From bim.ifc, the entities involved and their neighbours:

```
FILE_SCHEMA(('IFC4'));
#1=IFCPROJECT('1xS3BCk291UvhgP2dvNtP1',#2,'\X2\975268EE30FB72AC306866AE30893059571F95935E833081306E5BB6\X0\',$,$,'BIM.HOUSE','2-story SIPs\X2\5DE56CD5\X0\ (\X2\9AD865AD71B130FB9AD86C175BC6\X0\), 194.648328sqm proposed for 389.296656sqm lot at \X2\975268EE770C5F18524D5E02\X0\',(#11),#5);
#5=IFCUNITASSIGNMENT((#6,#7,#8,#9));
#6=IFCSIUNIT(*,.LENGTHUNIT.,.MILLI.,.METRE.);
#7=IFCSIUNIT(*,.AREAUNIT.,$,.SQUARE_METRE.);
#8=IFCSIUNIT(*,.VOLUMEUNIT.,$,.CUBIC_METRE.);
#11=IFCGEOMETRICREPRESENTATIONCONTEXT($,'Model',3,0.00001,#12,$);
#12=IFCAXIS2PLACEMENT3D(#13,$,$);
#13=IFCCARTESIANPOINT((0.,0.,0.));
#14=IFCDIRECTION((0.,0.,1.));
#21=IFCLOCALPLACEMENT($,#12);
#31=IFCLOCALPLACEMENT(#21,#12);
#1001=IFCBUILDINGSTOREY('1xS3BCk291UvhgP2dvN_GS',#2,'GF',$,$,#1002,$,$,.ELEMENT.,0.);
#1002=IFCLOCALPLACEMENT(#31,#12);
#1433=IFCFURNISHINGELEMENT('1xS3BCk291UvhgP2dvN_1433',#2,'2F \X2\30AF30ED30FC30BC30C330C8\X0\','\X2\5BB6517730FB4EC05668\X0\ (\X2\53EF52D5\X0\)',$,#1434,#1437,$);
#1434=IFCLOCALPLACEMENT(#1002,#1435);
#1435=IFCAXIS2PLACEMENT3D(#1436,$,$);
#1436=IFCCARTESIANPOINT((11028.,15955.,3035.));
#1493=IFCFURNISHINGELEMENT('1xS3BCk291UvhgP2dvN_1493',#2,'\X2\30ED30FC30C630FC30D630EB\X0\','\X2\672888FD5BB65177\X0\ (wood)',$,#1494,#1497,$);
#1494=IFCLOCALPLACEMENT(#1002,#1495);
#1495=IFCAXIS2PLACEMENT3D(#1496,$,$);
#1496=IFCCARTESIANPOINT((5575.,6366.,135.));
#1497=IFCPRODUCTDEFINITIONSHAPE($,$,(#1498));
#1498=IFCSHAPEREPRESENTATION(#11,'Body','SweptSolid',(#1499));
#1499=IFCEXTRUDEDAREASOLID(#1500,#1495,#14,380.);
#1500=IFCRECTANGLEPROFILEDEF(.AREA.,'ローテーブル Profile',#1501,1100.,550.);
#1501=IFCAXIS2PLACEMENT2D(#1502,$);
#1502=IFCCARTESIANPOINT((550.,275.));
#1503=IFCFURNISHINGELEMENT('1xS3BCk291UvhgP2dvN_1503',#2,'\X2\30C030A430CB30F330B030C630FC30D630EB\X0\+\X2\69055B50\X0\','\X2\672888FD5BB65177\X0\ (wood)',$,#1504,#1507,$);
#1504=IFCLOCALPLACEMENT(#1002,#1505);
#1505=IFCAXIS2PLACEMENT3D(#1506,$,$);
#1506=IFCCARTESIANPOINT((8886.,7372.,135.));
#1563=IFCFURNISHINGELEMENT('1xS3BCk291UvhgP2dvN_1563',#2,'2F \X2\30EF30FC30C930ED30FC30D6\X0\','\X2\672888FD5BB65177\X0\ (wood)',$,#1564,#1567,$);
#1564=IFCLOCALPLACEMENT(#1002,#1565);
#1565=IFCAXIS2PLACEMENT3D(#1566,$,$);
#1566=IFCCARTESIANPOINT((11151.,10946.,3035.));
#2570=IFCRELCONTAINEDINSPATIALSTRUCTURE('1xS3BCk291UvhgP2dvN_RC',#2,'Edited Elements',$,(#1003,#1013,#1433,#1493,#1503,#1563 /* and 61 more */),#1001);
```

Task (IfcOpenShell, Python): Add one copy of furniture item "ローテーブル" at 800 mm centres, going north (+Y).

```python
import numpy as np
import ifcopenshell
import ifcopenshell.api.geometry
import ifcopenshell.api.root
import ifcopenshell.util.element
import ifcopenshell.util.placement
import ifcopenshell.util.unit

model = ifcopenshell.open("bim.ifc")
unit_scale = ifcopenshell.util.unit.calculate_unit_scale(model)


def reuse_history(source, copy):
    """copy_class also copies each property set's owner history, people and application; keep the originals."""
    for rel in copy.IsDefinedBy:
        if rel.is_a("IfcRelDefinesByProperties") and (history := rel.RelatingPropertyDefinition.OwnerHistory):
            rel.RelatingPropertyDefinition.OwnerHistory = source.OwnerHistory
            ifcopenshell.util.element.remove_deep2(model, history)


source = model.by_guid("1xS3BCk291UvhgP2dvN_1493")
base = ifcopenshell.util.placement.get_local_placement(source.ObjectPlacement)
step = np.array([0.0, 1.0, 0.0]) * 0.8 / unit_scale

for i in range(1, 2):
    copy = ifcopenshell.api.root.copy_class(model, product=source)
    copy.Representation = ifcopenshell.util.element.copy_deep(
        model, source.Representation, exclude=["IfcGeometricRepresentationContext", "IfcRepresentationMap"]
    )
    reuse_history(source, copy)
    matrix = base.copy()
    matrix[:3, 3] += i * step
    print("added at", matrix[:3, 3].round(3) + 0.0)
    ifcopenshell.api.geometry.edit_object_placement(model, product=copy, matrix=matrix, is_si=False)

model.write("bim-out.ifc")
```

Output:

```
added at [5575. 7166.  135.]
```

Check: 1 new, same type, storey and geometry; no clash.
